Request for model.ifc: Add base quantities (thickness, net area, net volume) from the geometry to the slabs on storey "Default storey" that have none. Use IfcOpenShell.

First a look at what the model holds.

```python
import ifcopenshell
import ifcopenshell.util.element
import ifcopenshell.util.unit

model = ifcopenshell.open("model.ifc")
print(model.schema)
for unit_type in ("LENGTHUNIT", "AREAUNIT", "VOLUMEUNIT"):
    print(unit_type, ifcopenshell.util.unit.calculate_unit_scale(model, unit_type))
storey = next(s for s in model.by_type("IfcBuildingStorey") if s.Name == "Default storey")
slabs = [e for e in ifcopenshell.util.element.get_decomposition(storey) if e.is_a("IfcSlab")]
for e in sorted(slabs, key=lambda e: e.id()):
    print(e.id(), e.is_a(), e.Name, list(ifcopenshell.util.element.get_psets(e, qtos_only=True)), sep=" | ")
```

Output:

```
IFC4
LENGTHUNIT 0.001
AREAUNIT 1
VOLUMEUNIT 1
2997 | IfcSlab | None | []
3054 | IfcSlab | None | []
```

```python
import ifcopenshell
import ifcopenshell.api.pset
import ifcopenshell.geom
import ifcopenshell.util.element
import ifcopenshell.util.shape
import ifcopenshell.util.unit

model = ifcopenshell.open("model.ifc")
unit_scale = ifcopenshell.util.unit.calculate_unit_scale(model)
area_scale = ifcopenshell.util.unit.calculate_unit_scale(model, "AREAUNIT")
volume_scale = ifcopenshell.util.unit.calculate_unit_scale(model, "VOLUMEUNIT")
settings = ifcopenshell.geom.settings()

storey = next(s for s in model.by_type("IfcBuildingStorey") if s.Name == "Default storey")
slabs = [e for e in ifcopenshell.util.element.get_decomposition(storey) if e.is_a("IfcSlab")]

for e in sorted(slabs, key=lambda e: e.id()):
    if ifcopenshell.util.element.get_psets(e, qtos_only=True, should_inherit=False):
        continue
    # Geometry comes back in metres, in the element's own axes.
    shape = ifcopenshell.geom.create_shape(settings, e)
    values = {
        "Width": ifcopenshell.util.shape.get_z(shape.geometry) / unit_scale,
        "NetArea": ifcopenshell.util.shape.get_footprint_area(shape.geometry) / area_scale,
        "NetVolume": ifcopenshell.util.shape.get_volume(shape.geometry) / volume_scale,
    }
    qto = ifcopenshell.api.pset.add_qto(model, product=e, name="Qto_SlabBaseQuantities")
    ifcopenshell.api.pset.edit_qto(model, qto=qto, properties=values)
    print(e.id(), {k: round(v, 3) for k, v in values.items()})

model.write("model_v2.ifc")
```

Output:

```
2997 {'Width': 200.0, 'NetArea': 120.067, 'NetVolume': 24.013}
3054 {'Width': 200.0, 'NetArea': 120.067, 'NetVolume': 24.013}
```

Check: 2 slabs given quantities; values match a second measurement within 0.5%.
